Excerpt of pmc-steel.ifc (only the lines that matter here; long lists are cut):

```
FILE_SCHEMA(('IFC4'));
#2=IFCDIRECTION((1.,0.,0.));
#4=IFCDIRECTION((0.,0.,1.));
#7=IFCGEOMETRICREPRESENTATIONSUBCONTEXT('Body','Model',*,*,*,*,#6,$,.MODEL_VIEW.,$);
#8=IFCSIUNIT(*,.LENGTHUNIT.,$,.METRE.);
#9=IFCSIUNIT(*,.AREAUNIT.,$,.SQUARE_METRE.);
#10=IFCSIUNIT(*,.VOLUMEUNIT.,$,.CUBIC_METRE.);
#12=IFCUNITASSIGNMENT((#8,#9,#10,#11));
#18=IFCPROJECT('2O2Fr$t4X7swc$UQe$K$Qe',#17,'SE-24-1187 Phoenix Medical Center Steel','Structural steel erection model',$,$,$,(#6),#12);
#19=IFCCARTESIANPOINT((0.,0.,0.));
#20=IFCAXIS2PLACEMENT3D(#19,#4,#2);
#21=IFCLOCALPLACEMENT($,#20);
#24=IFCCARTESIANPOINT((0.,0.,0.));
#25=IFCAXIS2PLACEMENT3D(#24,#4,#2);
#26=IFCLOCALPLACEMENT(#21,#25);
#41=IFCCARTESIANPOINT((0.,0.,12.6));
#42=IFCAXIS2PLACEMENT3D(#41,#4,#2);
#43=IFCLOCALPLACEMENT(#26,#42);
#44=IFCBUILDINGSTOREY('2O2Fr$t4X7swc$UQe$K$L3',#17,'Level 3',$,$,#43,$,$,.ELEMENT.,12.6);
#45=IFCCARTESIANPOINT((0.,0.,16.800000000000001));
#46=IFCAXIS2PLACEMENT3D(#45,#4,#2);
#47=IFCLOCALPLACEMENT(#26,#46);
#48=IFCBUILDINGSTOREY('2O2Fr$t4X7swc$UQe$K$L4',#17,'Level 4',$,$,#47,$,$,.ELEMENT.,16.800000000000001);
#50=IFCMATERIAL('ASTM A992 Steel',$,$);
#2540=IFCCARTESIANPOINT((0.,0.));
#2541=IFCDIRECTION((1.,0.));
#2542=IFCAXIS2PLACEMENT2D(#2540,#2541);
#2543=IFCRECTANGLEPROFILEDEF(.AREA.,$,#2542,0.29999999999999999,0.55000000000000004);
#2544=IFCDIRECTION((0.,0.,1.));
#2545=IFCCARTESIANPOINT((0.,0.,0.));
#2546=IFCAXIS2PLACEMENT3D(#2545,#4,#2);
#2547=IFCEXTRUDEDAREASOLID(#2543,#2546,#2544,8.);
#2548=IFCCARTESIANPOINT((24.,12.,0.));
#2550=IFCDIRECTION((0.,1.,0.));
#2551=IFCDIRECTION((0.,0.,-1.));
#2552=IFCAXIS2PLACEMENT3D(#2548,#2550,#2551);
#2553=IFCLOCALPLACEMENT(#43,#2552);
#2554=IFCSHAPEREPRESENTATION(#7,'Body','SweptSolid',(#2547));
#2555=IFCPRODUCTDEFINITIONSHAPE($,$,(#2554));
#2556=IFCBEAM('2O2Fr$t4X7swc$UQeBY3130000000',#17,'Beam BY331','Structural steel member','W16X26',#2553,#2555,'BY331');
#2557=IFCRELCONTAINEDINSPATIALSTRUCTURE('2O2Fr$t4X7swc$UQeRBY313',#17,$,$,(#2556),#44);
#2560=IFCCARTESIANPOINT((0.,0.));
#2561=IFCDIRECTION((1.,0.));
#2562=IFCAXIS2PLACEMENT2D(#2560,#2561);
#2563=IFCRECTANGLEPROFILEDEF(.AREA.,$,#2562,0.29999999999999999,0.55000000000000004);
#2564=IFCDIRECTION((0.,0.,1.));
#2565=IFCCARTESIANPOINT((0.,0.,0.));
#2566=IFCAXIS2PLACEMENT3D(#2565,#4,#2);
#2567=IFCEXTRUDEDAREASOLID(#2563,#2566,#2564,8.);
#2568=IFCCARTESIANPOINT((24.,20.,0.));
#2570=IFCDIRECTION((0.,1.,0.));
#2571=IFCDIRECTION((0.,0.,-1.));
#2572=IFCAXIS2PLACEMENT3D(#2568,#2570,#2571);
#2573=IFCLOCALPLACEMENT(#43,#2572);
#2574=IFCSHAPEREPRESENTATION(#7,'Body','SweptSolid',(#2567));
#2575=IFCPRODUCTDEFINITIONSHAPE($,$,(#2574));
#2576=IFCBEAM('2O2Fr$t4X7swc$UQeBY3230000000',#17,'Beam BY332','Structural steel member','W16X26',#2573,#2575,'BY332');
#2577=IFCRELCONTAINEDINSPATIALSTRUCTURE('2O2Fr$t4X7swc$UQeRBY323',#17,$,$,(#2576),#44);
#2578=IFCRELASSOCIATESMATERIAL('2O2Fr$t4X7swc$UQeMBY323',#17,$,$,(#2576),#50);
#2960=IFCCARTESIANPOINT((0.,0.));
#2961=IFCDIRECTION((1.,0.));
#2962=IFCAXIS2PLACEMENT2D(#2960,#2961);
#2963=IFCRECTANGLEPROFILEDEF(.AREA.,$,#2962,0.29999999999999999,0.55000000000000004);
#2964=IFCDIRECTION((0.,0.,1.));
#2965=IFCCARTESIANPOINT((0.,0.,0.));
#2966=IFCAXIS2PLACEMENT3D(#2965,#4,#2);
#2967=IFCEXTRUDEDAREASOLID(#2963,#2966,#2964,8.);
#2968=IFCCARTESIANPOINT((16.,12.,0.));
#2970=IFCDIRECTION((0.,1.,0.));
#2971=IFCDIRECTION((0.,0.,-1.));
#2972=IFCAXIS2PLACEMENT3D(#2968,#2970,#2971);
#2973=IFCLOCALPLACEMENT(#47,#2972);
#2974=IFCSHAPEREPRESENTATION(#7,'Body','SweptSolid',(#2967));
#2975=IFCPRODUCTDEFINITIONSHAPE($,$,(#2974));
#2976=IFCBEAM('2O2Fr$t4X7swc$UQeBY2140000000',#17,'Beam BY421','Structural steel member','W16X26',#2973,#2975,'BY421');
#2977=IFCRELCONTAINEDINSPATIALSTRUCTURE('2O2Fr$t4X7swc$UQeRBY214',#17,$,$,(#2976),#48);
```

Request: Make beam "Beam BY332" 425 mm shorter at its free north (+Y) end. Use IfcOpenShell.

```python
import ifcopenshell
import ifcopenshell.util.representation

model = ifcopenshell.open("pmc-steel.ifc")

member = model.by_guid("2O2Fr$t4X7swc$UQeBY3230000000")
change = -0.425

# The extrusion runs towards the end named, so only its depth changes.
body = ifcopenshell.util.representation.get_representation(member, "Model", "Body")
solid = body.Items[0]
old_length = solid.Depth
solid.Depth += change

print(f"length {old_length:g} -> {solid.Depth:g}")

model.write("pmc-steel_v2.ifc")
```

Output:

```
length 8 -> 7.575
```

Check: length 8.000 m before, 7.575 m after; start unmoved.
